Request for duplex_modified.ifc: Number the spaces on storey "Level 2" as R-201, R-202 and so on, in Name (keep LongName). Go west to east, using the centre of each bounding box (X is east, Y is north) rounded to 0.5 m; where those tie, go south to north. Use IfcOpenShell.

First a look at what the model holds.

```python
import ifcopenshell
import ifcopenshell.util.element
import ifcopenshell.util.placement

model = ifcopenshell.open("duplex_modified.ifc")
print(model.schema)
storey = next(s for s in model.by_type("IfcBuildingStorey") if s.Name == "Level 2")
spaces = [e for e in ifcopenshell.util.element.get_decomposition(storey) if e.is_a("IfcSpace")]
for e in sorted(spaces, key=lambda e: e.id()):
    origin = ifcopenshell.util.placement.get_local_placement(e.ObjectPlacement)[:3, 3]
    print(e.id(), e.Name, e.LongName, origin.round(2) + 0.0, sep=" | ")
```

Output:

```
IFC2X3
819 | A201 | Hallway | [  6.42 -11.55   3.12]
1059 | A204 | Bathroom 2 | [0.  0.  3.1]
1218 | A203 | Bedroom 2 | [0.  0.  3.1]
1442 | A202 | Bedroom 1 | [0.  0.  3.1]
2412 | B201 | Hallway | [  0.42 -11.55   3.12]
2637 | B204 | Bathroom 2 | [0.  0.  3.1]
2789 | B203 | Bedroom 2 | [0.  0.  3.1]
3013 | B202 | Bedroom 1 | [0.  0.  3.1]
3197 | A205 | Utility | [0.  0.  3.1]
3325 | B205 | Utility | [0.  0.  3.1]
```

```python
import ifcopenshell
import ifcopenshell.geom
import ifcopenshell.util.element
import ifcopenshell.util.shape

model = ifcopenshell.open("duplex_modified.ifc")
settings = ifcopenshell.geom.settings()
settings.set("use-world-coords", True)


def centre(element):
    shape = ifcopenshell.geom.create_shape(settings, element)
    return ifcopenshell.util.shape.get_bbox_centroid(shape.geometry)


storey = next(s for s in model.by_type("IfcBuildingStorey") if s.Name == "Level 2")
spaces = [e for e in ifcopenshell.util.element.get_decomposition(storey) if e.is_a("IfcSpace")]

# Insertion points can sit at a corner or the storey origin, so sort by the geometry (in metres).
centres = {e: centre(e) for e in spaces}
spaces.sort(key=lambda e: (round(centres[e][0] / 0.5), centres[e][1]))

for i, e in enumerate(spaces, start=1):
    number = f"R-2{i:02d}"
    e.Name = number
    print(e.id(), number)

model.write("duplex_modified_rev.ifc")
```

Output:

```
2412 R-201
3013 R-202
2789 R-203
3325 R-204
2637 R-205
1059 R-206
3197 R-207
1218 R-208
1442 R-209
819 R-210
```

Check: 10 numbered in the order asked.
